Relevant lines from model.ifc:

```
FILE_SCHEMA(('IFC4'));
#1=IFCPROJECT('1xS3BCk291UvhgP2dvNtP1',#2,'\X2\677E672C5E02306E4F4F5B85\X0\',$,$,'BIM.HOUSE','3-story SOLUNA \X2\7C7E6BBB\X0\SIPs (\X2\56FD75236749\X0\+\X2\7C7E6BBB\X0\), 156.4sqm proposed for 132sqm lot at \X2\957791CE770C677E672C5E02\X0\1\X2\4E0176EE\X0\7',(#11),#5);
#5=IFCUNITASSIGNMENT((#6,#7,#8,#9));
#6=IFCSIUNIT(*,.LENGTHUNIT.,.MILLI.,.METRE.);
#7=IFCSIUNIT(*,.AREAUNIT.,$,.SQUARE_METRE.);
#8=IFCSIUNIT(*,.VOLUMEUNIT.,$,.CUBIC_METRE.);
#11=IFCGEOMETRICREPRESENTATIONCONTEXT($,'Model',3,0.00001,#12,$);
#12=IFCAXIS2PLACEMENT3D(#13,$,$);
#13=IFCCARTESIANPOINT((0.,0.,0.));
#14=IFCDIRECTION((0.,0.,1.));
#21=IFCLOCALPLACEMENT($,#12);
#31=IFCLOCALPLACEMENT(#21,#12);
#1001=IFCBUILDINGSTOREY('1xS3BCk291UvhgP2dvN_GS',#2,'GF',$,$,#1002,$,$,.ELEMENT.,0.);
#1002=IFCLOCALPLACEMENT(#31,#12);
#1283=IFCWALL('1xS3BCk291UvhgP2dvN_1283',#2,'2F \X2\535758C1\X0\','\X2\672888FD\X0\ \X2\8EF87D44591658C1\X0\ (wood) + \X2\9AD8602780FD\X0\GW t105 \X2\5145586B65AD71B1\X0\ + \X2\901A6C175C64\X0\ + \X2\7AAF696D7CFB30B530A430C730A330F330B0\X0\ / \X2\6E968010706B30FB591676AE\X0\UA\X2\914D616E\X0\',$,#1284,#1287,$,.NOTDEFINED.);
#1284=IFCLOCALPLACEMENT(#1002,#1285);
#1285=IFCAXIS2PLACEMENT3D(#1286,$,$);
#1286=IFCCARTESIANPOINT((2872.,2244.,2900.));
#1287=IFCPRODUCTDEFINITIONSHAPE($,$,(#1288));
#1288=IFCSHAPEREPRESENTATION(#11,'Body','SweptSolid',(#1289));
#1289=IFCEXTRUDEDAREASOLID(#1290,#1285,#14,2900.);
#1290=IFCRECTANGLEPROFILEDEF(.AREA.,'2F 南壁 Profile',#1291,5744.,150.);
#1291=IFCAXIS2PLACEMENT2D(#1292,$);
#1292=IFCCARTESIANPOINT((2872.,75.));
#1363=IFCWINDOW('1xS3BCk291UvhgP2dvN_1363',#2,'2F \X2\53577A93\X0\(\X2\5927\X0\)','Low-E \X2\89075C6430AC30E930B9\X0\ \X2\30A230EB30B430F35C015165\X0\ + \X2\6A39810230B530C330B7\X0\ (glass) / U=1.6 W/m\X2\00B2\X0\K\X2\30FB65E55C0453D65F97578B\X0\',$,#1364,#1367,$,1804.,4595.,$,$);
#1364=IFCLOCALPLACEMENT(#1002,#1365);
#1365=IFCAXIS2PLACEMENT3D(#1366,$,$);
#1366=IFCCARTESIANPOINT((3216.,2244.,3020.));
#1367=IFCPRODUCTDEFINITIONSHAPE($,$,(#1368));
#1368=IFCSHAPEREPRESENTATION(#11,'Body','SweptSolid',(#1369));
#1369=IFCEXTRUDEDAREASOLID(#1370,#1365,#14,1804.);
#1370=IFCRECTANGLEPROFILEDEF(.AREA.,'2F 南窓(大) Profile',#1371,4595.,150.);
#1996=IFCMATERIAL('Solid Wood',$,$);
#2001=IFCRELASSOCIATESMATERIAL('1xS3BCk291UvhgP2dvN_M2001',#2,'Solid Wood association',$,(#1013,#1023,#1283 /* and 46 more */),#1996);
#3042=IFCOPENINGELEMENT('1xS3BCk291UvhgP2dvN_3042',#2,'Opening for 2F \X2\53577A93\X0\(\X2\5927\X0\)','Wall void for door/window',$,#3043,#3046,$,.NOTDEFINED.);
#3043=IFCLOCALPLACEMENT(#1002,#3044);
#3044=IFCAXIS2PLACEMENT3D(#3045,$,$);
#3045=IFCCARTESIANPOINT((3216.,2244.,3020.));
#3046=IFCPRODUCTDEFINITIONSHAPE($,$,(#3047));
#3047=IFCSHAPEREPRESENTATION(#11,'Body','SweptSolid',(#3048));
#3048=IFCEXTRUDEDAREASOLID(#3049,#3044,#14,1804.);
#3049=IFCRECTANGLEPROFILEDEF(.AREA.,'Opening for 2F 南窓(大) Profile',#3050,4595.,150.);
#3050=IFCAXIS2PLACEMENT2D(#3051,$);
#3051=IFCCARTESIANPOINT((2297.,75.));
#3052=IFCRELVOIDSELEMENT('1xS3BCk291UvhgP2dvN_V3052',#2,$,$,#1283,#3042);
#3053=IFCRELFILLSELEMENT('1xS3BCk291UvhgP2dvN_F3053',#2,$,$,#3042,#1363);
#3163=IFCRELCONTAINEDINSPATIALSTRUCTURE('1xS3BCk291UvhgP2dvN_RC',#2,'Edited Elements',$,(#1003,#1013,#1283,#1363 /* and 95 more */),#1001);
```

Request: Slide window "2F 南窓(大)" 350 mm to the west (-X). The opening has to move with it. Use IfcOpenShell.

```python
import ifcopenshell
import ifcopenshell.api.geometry
import ifcopenshell.util.placement
import ifcopenshell.util.unit

model = ifcopenshell.open("model.ifc")
unit_scale = ifcopenshell.util.unit.calculate_unit_scale(model)

window = model.by_guid("1xS3BCk291UvhgP2dvN_1363")
opening = window.FillsVoids[0].RelatingOpeningElement
wall = opening.VoidsElements[0].RelatingBuildingElement

wall_matrix = ifcopenshell.util.placement.get_local_placement(wall.ObjectPlacement)
shift = wall_matrix[:3, 0] * -0.35 / unit_scale
before = ifcopenshell.util.placement.get_local_placement(window.ObjectPlacement)[:3, 3].copy()

# The window is not placed relative to its opening, so move both.
for product in (opening, window):
    matrix = ifcopenshell.util.placement.get_local_placement(product.ObjectPlacement)
    matrix[:3, 3] += shift
    ifcopenshell.api.geometry.edit_object_placement(model, product=product, matrix=matrix, is_si=False)

after = ifcopenshell.util.placement.get_local_placement(window.ObjectPlacement)[:3, 3]
print("window moved by", (after - before).round(3) + 0.0)

model.write("model_updated.ifc")
```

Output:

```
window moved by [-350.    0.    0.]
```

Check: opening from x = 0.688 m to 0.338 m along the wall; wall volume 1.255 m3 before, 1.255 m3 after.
